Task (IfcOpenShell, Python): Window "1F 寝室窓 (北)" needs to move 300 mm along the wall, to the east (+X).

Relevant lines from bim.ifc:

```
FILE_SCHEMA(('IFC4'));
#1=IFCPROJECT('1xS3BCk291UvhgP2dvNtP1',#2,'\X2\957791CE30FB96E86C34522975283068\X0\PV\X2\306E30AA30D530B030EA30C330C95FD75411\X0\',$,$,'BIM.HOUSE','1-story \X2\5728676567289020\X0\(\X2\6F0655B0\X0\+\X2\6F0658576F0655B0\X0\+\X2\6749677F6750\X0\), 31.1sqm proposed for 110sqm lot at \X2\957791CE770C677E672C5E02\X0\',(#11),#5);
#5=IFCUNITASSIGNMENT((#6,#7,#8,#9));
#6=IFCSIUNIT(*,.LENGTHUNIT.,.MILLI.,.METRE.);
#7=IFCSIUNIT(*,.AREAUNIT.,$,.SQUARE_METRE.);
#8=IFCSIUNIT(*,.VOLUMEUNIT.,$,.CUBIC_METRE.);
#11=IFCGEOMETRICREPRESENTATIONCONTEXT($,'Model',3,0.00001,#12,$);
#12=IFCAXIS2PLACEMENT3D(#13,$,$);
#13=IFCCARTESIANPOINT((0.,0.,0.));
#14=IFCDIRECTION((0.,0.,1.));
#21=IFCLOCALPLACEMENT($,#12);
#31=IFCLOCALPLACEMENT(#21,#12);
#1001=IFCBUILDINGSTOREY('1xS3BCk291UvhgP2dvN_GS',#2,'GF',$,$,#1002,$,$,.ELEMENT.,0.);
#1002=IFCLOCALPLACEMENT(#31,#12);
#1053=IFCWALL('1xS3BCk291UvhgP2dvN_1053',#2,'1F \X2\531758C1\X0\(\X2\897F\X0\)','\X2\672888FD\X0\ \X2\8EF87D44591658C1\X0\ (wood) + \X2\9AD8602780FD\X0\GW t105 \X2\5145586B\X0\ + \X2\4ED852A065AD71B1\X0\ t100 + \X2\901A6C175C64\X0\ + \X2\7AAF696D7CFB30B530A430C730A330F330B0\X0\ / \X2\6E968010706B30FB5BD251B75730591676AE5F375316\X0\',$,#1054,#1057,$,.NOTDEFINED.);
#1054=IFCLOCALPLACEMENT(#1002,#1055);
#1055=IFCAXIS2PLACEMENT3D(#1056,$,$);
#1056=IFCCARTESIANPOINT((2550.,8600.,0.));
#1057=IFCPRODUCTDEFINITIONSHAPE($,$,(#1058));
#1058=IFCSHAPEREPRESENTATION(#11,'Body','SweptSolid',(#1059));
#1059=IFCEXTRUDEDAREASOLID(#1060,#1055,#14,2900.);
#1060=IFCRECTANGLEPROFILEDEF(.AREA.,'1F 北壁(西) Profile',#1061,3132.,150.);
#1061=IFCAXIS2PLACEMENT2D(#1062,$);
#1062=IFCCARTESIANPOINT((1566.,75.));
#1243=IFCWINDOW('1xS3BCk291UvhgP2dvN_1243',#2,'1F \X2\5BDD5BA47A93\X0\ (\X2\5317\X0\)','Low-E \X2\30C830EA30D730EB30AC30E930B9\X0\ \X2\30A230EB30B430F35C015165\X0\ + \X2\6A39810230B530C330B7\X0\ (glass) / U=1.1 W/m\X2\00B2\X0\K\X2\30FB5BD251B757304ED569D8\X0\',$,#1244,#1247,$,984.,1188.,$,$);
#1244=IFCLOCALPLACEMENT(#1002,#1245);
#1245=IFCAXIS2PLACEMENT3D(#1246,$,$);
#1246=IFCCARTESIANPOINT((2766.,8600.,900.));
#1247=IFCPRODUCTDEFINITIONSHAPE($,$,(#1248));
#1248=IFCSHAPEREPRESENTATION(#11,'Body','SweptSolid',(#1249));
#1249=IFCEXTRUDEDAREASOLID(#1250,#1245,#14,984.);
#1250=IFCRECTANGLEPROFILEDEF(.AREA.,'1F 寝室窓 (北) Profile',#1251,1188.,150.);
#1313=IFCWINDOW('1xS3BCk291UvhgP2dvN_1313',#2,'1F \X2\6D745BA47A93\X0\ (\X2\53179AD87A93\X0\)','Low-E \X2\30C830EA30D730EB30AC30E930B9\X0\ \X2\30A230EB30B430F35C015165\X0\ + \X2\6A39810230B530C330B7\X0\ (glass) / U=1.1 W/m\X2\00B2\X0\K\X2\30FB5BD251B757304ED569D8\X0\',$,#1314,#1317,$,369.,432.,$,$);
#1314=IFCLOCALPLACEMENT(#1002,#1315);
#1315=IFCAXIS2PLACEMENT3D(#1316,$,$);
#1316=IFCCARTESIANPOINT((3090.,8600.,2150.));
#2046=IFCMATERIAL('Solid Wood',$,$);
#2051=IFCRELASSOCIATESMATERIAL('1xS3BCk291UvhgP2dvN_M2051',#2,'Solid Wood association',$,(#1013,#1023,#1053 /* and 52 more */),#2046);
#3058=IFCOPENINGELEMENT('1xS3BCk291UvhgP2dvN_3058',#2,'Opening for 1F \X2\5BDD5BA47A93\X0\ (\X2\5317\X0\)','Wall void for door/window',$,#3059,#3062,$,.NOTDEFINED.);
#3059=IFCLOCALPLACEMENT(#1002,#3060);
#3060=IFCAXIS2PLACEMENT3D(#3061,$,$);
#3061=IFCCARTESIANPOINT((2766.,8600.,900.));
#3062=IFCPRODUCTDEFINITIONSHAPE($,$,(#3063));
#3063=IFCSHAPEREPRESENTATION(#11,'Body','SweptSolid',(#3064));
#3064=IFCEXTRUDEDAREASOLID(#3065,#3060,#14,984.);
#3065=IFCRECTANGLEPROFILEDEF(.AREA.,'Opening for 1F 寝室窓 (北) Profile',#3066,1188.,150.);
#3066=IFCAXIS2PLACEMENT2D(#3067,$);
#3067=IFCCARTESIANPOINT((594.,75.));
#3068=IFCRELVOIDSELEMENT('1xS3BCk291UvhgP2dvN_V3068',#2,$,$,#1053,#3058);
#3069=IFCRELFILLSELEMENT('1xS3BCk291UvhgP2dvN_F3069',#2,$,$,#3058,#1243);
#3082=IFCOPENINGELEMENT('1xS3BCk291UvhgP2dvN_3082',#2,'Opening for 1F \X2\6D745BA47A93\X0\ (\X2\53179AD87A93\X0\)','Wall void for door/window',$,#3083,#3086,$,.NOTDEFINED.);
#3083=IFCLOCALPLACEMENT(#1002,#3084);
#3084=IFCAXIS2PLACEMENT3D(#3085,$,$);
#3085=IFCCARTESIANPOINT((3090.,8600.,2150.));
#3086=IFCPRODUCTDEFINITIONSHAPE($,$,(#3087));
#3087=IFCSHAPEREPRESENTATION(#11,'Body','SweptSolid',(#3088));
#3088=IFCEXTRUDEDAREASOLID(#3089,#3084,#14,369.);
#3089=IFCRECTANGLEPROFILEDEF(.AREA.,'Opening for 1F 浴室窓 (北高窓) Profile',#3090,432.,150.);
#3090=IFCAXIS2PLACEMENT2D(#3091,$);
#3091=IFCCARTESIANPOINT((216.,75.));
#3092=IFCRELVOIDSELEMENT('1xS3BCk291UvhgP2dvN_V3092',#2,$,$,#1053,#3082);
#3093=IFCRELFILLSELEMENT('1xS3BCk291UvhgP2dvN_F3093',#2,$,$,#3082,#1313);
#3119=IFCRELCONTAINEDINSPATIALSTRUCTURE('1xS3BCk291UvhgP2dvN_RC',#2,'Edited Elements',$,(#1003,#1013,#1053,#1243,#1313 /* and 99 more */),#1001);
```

```python
import ifcopenshell
import ifcopenshell.api.geometry
import ifcopenshell.util.placement
import ifcopenshell.util.unit

model = ifcopenshell.open("bim.ifc")
unit_scale = ifcopenshell.util.unit.calculate_unit_scale(model)

window = model.by_guid("1xS3BCk291UvhgP2dvN_1243")
opening = window.FillsVoids[0].RelatingOpeningElement
wall = opening.VoidsElements[0].RelatingBuildingElement

wall_matrix = ifcopenshell.util.placement.get_local_placement(wall.ObjectPlacement)
shift = wall_matrix[:3, 0] * 0.3 / unit_scale
before = ifcopenshell.util.placement.get_local_placement(window.ObjectPlacement)[:3, 3].copy()

# The window is not placed relative to its opening, so move both.
for product in (opening, window):
    matrix = ifcopenshell.util.placement.get_local_placement(product.ObjectPlacement)
    matrix[:3, 3] += shift
    ifcopenshell.api.geometry.edit_object_placement(model, product=product, matrix=matrix, is_si=False)

after = ifcopenshell.util.placement.get_local_placement(window.ObjectPlacement)[:3, 3]
print("window moved by", (after - before).round(3) + 0.0)

model.write("bim_updated.ifc")
```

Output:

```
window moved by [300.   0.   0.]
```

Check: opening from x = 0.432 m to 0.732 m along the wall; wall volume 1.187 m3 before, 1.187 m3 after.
